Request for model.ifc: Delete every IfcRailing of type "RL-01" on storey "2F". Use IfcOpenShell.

First a look at what the model holds.

```python
import ifcopenshell
import ifcopenshell.util.element

model = ifcopenshell.open("model.ifc")
print(model.schema)
storey = next(s for s in model.by_type("IfcBuildingStorey") if s.Name == "2F")
railings = [e for e in ifcopenshell.util.element.get_decomposition(storey) if e.is_a("IfcRailing")]
seen = {}
for e in railings:
    element_type = ifcopenshell.util.element.get_type(e)
    name = element_type.Name if element_type not in (None, e) else None
    seen[name] = seen.get(name, 0) + 1
for name, count in sorted(seen.items(), key=str):
    print(count, "x", name)
```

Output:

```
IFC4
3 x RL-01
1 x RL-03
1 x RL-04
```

```python
import ifcopenshell
import ifcopenshell.api.root
import ifcopenshell.util.element

model = ifcopenshell.open("model.ifc")

storey = next(s for s in model.by_type("IfcBuildingStorey") if s.Name == "2F")
railings = [e for e in ifcopenshell.util.element.get_decomposition(storey) if e.is_a("IfcRailing")]
targets = [e for e in railings if (t := ifcopenshell.util.element.get_type(e)) not in (None, e) and t.Name == "RL-01"]

for e in targets:
    ifcopenshell.api.root.remove_product(model, product=e)
print(len(targets), "removed")

model.write("model_rev.ifc")
```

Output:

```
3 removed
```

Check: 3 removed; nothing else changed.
